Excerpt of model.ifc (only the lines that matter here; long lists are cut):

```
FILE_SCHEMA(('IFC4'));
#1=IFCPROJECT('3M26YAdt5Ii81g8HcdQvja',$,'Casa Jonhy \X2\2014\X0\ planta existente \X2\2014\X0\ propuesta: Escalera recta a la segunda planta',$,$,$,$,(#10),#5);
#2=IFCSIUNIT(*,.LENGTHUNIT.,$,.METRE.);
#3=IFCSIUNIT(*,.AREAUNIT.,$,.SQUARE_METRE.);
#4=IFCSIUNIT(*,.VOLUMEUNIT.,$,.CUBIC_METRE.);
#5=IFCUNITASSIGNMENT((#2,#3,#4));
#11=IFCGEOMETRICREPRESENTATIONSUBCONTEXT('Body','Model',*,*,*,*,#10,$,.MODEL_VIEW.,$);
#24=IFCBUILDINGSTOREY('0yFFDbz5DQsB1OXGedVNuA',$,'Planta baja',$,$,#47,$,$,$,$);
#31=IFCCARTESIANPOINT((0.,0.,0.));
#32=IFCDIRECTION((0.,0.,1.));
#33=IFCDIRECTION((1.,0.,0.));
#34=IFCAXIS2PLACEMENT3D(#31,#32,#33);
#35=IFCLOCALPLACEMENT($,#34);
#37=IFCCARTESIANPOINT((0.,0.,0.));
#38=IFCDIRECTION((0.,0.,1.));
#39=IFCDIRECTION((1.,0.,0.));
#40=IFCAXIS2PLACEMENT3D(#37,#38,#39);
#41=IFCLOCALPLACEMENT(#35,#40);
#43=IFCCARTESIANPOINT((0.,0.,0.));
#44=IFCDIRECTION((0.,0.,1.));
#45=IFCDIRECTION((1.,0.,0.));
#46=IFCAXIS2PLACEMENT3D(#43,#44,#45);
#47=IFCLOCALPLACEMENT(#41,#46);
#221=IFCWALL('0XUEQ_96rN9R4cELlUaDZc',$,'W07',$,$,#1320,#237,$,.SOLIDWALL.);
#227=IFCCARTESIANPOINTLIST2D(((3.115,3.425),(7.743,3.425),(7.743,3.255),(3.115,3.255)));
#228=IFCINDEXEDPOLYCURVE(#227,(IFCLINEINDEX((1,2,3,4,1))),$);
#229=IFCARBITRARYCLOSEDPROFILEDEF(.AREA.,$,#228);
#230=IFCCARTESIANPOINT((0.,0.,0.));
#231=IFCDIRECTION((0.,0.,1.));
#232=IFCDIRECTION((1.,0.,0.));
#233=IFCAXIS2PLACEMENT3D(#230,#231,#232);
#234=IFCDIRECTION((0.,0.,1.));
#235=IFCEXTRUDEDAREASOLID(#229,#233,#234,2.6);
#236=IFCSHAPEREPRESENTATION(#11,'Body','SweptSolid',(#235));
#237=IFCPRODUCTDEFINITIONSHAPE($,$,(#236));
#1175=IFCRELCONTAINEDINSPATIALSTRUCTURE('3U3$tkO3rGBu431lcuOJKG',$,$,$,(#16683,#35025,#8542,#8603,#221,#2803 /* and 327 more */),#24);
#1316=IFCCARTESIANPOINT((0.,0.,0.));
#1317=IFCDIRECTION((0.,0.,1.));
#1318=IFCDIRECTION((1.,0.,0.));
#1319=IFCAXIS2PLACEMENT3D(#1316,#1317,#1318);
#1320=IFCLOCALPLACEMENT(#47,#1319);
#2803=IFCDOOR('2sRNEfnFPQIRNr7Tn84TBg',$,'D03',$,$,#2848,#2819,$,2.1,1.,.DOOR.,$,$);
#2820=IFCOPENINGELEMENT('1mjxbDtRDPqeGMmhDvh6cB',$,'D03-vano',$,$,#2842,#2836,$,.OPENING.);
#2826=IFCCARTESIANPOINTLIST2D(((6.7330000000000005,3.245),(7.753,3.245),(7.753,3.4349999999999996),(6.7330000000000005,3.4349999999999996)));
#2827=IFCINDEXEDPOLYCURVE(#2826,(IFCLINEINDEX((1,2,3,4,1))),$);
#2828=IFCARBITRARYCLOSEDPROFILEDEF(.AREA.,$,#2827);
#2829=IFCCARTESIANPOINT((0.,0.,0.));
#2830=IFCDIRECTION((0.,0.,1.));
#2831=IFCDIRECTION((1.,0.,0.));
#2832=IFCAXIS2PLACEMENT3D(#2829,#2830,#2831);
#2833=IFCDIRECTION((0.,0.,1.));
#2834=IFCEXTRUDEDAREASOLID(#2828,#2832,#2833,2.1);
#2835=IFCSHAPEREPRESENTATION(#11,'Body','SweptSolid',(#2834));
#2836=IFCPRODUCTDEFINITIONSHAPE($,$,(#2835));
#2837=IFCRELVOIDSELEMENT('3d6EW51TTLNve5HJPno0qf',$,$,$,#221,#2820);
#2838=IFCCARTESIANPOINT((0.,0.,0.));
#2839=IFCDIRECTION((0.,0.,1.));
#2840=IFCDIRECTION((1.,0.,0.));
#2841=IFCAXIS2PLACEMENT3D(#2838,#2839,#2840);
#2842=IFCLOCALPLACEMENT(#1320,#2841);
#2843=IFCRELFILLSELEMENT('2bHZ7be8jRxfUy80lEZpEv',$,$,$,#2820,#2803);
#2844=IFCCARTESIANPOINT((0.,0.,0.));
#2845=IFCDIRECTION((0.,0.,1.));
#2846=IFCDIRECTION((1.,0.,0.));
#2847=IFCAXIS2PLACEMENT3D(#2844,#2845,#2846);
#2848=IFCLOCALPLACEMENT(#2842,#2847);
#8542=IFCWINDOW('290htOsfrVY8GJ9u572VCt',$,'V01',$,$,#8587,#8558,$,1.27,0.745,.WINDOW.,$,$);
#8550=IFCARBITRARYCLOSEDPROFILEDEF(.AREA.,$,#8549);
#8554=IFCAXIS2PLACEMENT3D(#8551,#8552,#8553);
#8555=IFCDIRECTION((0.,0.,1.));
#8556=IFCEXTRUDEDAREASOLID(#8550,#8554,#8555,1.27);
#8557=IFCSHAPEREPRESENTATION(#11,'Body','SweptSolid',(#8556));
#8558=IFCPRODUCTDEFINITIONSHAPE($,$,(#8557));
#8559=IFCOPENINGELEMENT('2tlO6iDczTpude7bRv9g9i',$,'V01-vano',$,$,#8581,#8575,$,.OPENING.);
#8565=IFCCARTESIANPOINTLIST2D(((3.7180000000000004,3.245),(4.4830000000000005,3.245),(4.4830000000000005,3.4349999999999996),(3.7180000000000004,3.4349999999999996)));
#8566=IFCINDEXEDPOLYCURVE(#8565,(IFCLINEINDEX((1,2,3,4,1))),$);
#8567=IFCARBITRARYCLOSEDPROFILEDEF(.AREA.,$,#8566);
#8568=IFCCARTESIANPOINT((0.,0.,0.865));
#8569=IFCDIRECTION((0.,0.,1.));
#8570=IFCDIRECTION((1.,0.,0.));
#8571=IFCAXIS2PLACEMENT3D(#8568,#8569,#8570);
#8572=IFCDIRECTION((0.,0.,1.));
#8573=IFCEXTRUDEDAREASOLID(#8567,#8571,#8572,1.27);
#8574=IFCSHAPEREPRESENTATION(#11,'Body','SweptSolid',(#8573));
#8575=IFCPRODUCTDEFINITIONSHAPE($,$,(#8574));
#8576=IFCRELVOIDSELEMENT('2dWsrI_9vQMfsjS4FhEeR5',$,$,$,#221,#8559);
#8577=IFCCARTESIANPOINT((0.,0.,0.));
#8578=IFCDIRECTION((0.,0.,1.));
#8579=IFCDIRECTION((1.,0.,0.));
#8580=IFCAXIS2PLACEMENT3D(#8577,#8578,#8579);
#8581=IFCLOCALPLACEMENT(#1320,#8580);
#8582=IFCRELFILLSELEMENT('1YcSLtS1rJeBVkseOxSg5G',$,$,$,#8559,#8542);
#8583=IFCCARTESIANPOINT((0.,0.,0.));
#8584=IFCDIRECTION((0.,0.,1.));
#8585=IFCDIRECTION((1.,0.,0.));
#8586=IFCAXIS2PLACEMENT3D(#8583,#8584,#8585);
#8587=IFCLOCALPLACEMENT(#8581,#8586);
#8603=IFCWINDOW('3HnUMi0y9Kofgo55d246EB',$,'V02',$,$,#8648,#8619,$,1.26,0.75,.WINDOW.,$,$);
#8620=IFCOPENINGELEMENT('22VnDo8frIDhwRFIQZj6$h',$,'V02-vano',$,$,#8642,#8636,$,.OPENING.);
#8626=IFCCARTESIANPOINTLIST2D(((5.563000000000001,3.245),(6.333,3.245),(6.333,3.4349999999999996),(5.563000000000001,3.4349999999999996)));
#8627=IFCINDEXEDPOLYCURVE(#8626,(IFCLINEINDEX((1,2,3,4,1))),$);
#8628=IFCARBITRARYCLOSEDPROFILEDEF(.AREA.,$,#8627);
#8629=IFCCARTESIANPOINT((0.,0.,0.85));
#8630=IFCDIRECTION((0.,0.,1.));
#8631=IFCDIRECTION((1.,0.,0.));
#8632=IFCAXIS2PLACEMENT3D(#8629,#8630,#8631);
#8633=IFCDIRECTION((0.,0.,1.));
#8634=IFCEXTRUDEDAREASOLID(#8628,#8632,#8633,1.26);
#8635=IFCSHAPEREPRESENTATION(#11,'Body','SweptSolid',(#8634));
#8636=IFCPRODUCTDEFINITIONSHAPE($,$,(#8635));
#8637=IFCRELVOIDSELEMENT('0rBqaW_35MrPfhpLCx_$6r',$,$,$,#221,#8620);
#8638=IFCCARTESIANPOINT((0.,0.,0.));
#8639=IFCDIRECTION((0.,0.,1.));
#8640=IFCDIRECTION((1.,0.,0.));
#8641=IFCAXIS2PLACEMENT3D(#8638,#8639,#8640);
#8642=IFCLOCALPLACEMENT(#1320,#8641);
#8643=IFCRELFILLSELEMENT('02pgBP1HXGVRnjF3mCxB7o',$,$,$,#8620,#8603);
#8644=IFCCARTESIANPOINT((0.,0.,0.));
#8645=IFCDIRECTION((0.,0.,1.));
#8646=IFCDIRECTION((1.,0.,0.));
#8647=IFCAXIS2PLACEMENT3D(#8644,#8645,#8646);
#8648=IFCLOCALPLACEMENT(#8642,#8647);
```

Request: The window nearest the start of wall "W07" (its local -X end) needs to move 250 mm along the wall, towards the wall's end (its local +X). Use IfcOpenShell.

```python
import ifcopenshell
import ifcopenshell.api.geometry
import ifcopenshell.util.placement
import ifcopenshell.util.unit

model = ifcopenshell.open("model.ifc")
unit_scale = ifcopenshell.util.unit.calculate_unit_scale(model)

window = model.by_guid("290htOsfrVY8GJ9u572VCt")
opening = window.FillsVoids[0].RelatingOpeningElement
wall = opening.VoidsElements[0].RelatingBuildingElement

wall_matrix = ifcopenshell.util.placement.get_local_placement(wall.ObjectPlacement)
shift = wall_matrix[:3, 0] * 0.25 / unit_scale
before = ifcopenshell.util.placement.get_local_placement(window.ObjectPlacement)[:3, 3].copy()

# The window is placed relative to its opening, so it follows when the opening moves.
matrix = ifcopenshell.util.placement.get_local_placement(opening.ObjectPlacement)
matrix[:3, 3] += shift
ifcopenshell.api.geometry.edit_object_placement(
    model, product=opening, matrix=matrix, is_si=False, should_transform_children=True
)

after = ifcopenshell.util.placement.get_local_placement(window.ObjectPlacement)[:3, 3]
print("window moved by", (after - before).round(3) + 0.0)

model.write("model_edited.ifc")
```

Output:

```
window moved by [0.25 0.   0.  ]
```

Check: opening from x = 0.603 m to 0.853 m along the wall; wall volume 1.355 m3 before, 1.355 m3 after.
